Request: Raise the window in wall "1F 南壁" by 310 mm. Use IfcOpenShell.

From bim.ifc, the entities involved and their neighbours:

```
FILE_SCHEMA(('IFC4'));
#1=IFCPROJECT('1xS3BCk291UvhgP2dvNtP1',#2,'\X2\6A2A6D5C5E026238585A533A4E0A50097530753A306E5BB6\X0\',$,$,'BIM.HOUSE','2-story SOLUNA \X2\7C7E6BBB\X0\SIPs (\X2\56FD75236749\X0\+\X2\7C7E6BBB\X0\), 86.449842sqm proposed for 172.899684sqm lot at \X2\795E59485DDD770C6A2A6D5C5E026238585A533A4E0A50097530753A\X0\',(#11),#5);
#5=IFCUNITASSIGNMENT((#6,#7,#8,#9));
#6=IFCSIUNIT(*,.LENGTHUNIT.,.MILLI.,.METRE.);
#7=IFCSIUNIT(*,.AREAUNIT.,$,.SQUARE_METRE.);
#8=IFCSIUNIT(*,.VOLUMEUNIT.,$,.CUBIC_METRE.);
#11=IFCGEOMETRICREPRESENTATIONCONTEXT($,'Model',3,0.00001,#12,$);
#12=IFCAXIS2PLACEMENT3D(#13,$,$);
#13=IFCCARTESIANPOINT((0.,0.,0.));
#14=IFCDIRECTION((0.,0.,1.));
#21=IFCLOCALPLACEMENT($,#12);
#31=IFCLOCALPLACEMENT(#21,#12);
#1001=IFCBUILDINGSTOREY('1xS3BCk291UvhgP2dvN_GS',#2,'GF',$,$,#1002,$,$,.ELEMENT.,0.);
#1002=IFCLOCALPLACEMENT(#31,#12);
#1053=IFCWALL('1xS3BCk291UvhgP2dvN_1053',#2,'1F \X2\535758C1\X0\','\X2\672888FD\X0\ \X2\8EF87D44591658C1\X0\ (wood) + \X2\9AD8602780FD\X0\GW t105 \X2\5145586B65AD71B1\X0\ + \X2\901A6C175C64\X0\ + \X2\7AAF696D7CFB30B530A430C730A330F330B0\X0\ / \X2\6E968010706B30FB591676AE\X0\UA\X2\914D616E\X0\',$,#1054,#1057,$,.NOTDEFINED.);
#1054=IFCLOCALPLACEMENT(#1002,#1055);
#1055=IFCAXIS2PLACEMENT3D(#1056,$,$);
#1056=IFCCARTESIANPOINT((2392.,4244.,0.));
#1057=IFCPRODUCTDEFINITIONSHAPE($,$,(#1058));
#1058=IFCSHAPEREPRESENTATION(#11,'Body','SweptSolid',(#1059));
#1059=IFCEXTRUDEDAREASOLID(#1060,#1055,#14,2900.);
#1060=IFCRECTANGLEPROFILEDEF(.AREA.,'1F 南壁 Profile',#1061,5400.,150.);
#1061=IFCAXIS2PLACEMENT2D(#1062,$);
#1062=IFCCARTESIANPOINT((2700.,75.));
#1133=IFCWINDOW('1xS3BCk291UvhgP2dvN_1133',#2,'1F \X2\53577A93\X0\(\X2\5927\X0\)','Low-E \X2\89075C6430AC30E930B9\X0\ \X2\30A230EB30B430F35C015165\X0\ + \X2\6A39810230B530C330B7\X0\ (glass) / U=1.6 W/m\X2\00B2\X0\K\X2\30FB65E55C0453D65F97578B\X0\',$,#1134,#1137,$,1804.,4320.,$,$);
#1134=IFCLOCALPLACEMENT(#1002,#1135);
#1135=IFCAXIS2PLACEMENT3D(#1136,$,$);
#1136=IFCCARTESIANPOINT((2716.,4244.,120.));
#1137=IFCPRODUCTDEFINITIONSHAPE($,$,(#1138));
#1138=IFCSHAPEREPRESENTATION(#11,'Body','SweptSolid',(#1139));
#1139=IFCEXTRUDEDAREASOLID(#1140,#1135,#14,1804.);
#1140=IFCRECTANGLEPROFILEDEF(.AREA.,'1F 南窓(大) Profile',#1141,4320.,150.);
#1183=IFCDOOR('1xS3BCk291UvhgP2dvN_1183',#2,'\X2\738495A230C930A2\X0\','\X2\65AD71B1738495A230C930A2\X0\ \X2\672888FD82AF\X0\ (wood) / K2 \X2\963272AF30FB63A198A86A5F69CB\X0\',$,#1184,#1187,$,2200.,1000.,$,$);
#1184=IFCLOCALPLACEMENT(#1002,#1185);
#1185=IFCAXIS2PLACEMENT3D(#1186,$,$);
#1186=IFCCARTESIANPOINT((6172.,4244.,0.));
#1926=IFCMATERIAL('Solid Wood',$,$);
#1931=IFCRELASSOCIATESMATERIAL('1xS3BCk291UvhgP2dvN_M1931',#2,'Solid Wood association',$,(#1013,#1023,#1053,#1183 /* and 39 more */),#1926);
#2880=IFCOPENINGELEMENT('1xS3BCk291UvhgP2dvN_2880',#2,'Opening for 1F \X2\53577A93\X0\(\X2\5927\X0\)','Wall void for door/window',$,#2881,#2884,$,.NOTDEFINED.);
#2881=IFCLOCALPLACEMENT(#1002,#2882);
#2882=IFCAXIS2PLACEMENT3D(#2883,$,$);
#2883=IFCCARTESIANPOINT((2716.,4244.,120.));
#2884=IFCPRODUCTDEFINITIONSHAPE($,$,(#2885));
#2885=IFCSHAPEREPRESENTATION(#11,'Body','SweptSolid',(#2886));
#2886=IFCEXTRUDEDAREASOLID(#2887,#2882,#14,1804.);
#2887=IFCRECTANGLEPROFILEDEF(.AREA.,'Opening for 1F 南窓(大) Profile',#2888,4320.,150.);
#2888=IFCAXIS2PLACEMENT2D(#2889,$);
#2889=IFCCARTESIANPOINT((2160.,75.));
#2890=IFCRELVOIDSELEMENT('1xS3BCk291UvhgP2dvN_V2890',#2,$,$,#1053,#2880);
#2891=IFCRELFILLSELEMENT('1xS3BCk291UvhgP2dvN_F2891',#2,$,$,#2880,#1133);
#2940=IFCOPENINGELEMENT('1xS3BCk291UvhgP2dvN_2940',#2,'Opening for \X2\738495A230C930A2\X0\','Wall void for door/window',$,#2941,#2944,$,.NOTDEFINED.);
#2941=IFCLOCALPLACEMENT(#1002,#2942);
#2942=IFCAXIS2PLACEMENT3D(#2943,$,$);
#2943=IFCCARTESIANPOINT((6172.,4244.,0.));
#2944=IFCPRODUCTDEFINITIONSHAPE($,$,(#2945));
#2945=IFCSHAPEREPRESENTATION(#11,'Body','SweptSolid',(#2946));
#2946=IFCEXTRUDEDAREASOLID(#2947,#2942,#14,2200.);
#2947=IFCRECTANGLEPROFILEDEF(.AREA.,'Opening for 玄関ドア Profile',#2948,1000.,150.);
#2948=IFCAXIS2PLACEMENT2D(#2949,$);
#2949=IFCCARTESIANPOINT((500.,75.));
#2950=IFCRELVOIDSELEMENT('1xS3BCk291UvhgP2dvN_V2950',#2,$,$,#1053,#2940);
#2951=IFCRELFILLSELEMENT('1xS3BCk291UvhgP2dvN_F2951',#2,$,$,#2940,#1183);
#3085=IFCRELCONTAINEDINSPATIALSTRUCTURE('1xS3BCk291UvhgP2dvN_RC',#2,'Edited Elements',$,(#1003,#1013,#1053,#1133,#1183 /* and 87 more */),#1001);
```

```python
import numpy as np
import ifcopenshell
import ifcopenshell.api.geometry
import ifcopenshell.util.placement
import ifcopenshell.util.unit

model = ifcopenshell.open("bim.ifc")
unit_scale = ifcopenshell.util.unit.calculate_unit_scale(model)

window = model.by_guid("1xS3BCk291UvhgP2dvN_1133")
opening = window.FillsVoids[0].RelatingOpeningElement
dz = 0.31 / unit_scale

shift = np.array([0.0, 0.0, dz])
# The window is not placed relative to its opening, so move both.
for product in (opening, window):
    matrix = ifcopenshell.util.placement.get_local_placement(product.ObjectPlacement)
    matrix[:3, 3] += shift
    ifcopenshell.api.geometry.edit_object_placement(model, product=product, matrix=matrix, is_si=False)

print(f"moved by {dz * unit_scale:+.3f} m")

model.write("bim_edited.ifc")
```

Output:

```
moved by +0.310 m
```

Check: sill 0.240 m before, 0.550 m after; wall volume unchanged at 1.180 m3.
